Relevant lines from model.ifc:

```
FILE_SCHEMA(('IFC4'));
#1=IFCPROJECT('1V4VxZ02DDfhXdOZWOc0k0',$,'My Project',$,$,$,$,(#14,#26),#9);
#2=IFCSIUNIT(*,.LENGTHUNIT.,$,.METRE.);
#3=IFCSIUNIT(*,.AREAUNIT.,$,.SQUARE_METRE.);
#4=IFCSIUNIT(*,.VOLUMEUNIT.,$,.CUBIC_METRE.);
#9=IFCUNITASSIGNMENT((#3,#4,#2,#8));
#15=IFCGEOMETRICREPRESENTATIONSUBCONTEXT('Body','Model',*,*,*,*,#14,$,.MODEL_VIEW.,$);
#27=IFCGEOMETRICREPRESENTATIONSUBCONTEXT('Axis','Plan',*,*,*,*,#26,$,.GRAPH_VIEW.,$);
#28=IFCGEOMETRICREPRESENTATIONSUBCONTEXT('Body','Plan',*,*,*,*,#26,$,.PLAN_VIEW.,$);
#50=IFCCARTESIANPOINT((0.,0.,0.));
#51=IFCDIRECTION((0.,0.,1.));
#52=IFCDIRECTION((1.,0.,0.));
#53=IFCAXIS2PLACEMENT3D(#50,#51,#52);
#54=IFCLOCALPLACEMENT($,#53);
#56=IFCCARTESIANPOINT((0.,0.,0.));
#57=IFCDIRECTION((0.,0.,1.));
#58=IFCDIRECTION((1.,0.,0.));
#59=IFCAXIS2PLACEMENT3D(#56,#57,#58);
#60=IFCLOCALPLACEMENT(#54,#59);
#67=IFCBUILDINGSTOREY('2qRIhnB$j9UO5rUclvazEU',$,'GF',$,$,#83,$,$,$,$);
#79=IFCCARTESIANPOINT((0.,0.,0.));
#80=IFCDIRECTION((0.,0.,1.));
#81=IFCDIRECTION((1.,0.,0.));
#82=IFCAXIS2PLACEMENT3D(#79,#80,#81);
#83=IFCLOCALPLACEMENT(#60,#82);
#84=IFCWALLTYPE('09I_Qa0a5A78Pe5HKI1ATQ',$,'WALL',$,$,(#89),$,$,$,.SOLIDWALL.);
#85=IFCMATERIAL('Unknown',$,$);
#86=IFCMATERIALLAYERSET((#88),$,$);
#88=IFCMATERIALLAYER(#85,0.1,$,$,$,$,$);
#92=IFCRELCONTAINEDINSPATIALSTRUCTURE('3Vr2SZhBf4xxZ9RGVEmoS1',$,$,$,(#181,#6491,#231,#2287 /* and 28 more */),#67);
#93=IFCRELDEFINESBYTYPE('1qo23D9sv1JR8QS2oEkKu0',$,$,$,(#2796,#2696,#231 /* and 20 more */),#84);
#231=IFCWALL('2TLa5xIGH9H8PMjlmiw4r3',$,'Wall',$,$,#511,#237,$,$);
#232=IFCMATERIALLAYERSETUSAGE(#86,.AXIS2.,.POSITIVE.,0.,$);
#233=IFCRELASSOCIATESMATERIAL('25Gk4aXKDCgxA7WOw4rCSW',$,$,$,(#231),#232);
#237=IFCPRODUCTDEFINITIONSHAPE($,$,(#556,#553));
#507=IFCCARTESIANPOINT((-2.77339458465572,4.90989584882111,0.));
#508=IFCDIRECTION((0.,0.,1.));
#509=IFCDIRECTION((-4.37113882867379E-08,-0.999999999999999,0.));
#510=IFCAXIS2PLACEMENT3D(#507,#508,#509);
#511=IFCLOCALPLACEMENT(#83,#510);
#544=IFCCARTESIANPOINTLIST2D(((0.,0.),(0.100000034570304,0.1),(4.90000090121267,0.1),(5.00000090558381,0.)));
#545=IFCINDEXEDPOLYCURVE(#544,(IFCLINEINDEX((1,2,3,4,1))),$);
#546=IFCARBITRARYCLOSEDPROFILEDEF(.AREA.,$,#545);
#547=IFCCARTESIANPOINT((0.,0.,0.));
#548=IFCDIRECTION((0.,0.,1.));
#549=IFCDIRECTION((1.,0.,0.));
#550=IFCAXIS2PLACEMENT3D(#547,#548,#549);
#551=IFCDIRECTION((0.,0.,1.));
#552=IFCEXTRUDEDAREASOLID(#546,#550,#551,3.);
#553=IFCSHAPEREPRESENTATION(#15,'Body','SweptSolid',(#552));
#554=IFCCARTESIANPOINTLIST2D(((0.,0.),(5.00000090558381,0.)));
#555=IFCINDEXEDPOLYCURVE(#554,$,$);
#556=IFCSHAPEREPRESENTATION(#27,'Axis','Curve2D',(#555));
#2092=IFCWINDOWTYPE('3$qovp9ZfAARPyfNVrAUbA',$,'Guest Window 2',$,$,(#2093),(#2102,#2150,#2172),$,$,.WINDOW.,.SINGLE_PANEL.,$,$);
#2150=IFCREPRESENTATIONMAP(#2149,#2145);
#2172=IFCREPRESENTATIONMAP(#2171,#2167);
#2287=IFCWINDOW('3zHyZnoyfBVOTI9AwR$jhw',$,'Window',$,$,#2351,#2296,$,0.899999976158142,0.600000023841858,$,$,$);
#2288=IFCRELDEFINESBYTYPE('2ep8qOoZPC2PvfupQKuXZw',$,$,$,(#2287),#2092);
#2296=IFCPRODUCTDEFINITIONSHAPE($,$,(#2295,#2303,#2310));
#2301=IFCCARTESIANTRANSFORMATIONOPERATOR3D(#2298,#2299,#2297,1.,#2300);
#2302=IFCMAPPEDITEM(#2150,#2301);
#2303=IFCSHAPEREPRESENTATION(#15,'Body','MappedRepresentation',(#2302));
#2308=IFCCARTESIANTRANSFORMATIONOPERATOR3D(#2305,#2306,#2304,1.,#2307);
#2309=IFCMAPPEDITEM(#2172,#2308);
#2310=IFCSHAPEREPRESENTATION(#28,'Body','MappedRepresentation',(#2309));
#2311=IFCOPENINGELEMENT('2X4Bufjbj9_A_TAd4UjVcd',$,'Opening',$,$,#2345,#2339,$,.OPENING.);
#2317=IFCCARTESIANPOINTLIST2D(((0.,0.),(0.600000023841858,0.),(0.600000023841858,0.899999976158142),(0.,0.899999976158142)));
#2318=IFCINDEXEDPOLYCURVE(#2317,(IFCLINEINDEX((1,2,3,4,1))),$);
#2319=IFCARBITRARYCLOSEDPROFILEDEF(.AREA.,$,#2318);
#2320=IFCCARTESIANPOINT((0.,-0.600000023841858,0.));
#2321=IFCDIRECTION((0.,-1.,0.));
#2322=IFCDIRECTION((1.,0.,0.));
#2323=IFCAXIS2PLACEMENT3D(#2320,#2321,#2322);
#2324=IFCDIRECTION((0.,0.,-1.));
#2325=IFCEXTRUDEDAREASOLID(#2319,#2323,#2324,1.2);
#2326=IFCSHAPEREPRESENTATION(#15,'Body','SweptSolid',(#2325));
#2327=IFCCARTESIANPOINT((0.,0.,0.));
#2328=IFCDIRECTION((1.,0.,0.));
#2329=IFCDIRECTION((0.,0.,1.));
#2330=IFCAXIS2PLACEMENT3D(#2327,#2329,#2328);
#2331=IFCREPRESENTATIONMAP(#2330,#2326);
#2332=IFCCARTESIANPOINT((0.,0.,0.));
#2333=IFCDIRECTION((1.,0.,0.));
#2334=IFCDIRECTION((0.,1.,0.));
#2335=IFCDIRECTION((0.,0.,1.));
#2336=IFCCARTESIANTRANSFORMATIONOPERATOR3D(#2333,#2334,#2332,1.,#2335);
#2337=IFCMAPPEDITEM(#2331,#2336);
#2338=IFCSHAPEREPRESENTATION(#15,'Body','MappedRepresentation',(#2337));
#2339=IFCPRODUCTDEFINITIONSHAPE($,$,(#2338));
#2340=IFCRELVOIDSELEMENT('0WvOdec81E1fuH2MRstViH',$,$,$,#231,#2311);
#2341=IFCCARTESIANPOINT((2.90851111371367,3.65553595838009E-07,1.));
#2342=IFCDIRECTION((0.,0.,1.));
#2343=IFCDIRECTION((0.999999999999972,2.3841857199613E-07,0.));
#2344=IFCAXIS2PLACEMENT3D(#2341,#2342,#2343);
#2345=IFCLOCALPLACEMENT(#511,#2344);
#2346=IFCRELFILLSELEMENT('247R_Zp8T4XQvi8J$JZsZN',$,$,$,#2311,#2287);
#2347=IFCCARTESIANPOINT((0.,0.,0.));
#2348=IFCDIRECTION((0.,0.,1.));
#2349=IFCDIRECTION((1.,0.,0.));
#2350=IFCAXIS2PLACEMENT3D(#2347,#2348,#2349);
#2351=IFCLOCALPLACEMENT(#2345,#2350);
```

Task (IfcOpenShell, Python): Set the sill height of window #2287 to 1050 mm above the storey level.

```python
import numpy as np
import ifcopenshell
import ifcopenshell.api.geometry
import ifcopenshell.geom
import ifcopenshell.util.element
import ifcopenshell.util.placement
import ifcopenshell.util.shape
import ifcopenshell.util.unit

model = ifcopenshell.open("model.ifc")
unit_scale = ifcopenshell.util.unit.calculate_unit_scale(model)

window = model.by_id(2287)
opening = window.FillsVoids[0].RelatingOpeningElement
storey = ifcopenshell.util.element.get_container(window, ifc_class="IfcBuildingStorey")
level = ifcopenshell.util.placement.get_local_placement(storey.ObjectPlacement)[2, 3]

# The opening's origin need not be at the sill, so measure its lowest point.
shape = ifcopenshell.geom.create_shape(ifcopenshell.geom.settings(), opening)
bottom = ifcopenshell.util.shape.get_shape_bottom_elevation(shape, shape.geometry) / unit_scale
dz = level + 1.05 - bottom

shift = np.array([0.0, 0.0, dz])
# The window is placed relative to its opening, so it follows when the opening moves.
matrix = ifcopenshell.util.placement.get_local_placement(opening.ObjectPlacement)
matrix[:3, 3] += shift
ifcopenshell.api.geometry.edit_object_placement(
    model, product=opening, matrix=matrix, is_si=False, should_transform_children=True
)

print(f"moved by {dz * unit_scale:+.3f} m")

model.write("model_v2.ifc")
```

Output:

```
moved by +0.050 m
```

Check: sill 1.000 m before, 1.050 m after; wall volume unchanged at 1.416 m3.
